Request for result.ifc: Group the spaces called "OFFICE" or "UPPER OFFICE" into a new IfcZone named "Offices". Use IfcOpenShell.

First a look at what the model holds.

```python
import ifcopenshell

model = ifcopenshell.open("result.ifc")
print(model.schema)
seen = {}
for space in model.by_type("IfcSpace"):
    seen[space.Name] = seen.get(space.Name, 0) + 1
for name, count in sorted(seen.items(), key=str):
    print(count, "x", name)
print("zones:", [z.Name for z in model.by_type("IfcZone")][:20])
```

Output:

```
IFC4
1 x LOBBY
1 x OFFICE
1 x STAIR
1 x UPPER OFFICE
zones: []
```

```python
import ifcopenshell
import ifcopenshell.api.group
import ifcopenshell.api.root

model = ifcopenshell.open("result.ifc")

names = {"OFFICE", "UPPER OFFICE"}
spaces = [s for s in model.by_type("IfcSpace") if s.Name in names]

zone = ifcopenshell.api.root.create_entity(model, ifc_class="IfcZone", name="Offices")
ifcopenshell.api.group.assign_group(model, products=spaces, group=zone)
print(len(spaces), "spaces in", zone.Name)

model.write("result_v2.ifc")
```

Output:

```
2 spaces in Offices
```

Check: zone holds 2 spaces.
